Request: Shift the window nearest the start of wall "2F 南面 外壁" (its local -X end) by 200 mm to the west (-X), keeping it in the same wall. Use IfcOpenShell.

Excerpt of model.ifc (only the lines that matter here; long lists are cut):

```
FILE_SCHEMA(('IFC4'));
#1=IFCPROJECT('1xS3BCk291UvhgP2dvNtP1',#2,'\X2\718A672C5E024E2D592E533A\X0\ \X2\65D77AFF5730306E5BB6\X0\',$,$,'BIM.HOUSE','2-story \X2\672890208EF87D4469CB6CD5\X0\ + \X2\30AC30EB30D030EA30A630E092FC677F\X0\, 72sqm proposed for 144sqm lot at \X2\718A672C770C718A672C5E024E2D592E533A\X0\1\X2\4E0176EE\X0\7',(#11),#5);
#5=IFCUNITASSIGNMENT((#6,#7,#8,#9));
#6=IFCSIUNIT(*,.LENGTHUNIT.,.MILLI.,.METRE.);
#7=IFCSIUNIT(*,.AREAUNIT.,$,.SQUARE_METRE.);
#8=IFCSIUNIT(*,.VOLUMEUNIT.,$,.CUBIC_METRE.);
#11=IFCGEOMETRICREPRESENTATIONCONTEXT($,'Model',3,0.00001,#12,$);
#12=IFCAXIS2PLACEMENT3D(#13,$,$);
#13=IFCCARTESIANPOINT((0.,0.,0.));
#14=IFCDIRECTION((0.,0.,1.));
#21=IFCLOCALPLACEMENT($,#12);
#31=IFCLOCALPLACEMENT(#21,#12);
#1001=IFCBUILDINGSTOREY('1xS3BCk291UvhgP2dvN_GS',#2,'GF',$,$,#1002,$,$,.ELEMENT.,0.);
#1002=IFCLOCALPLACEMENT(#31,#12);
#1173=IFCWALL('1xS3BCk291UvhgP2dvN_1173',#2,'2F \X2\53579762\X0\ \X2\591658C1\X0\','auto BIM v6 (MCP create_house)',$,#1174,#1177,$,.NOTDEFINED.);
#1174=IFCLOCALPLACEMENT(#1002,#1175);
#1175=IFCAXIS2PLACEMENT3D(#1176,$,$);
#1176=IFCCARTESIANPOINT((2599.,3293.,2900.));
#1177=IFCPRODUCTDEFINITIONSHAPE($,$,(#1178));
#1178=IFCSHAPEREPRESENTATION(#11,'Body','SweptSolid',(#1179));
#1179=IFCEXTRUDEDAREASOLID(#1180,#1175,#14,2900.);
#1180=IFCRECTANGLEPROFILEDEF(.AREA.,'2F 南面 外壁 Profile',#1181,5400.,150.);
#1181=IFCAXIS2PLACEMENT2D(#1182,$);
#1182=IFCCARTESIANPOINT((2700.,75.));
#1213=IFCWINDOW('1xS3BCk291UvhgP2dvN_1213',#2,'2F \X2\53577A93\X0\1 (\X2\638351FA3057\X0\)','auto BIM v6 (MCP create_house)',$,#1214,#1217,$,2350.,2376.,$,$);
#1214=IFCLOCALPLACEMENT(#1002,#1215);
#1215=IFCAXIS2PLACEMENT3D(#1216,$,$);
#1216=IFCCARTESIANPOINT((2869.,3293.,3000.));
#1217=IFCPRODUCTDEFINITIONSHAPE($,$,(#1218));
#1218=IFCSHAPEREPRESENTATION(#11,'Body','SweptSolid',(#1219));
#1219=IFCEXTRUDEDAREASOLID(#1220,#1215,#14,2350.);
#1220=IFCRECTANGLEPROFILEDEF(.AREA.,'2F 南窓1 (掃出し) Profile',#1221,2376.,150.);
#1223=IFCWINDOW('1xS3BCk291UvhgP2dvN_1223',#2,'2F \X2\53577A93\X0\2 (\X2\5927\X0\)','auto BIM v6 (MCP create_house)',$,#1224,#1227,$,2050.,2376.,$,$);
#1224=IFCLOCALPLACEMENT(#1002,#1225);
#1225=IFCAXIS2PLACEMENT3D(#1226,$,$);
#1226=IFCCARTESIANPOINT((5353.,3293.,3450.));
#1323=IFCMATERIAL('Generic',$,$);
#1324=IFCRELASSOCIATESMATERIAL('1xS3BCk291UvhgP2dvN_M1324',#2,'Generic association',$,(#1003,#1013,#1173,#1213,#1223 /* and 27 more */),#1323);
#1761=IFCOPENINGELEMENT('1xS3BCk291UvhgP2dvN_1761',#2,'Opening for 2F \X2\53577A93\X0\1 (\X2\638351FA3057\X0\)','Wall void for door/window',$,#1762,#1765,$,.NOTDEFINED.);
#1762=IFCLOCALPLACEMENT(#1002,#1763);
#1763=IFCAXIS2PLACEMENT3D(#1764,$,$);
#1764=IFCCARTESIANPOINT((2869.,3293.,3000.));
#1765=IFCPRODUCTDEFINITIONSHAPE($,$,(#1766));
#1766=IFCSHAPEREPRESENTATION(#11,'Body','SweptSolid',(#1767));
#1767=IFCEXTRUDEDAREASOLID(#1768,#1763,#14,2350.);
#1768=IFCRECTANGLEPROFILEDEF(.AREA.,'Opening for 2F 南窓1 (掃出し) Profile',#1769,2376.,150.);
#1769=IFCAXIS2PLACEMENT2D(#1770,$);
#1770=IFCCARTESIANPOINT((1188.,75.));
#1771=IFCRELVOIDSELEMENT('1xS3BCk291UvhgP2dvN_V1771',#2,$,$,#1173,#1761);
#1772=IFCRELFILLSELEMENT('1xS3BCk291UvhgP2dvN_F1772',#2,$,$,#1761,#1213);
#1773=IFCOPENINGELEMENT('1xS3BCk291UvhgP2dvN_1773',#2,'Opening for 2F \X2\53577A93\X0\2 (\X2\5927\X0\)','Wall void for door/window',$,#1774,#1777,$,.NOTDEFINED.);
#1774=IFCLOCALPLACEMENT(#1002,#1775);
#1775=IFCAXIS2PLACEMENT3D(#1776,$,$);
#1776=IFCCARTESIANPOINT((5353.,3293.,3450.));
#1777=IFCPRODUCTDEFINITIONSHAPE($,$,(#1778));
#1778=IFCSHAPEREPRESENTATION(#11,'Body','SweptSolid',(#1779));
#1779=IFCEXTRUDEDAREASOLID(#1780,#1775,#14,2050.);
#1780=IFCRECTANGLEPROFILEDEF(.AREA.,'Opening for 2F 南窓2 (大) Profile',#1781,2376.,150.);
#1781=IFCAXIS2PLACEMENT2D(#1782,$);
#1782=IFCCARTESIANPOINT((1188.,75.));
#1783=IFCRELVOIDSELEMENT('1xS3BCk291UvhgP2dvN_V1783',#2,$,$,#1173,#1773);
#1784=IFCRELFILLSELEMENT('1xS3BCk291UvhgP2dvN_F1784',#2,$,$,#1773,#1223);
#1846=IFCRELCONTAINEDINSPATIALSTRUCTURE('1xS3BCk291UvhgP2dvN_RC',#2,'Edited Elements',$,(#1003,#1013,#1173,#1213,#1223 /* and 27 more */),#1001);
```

```python
import ifcopenshell
import ifcopenshell.api.geometry
import ifcopenshell.util.placement

model = ifcopenshell.open("model.ifc")

window = model.by_guid("1xS3BCk291UvhgP2dvN_1213")
opening = window.FillsVoids[0].RelatingOpeningElement
wall = opening.VoidsElements[0].RelatingBuildingElement

wall_matrix = ifcopenshell.util.placement.get_local_placement(wall.ObjectPlacement)
shift = wall_matrix[:3, 0] * -200.0
before = ifcopenshell.util.placement.get_local_placement(window.ObjectPlacement)[:3, 3].copy()

# The window is not placed relative to its opening, so move both.
for product in (opening, window):
    matrix = ifcopenshell.util.placement.get_local_placement(product.ObjectPlacement)
    matrix[:3, 3] += shift
    ifcopenshell.api.geometry.edit_object_placement(model, product=product, matrix=matrix, is_si=False)

after = ifcopenshell.util.placement.get_local_placement(window.ObjectPlacement)[:3, 3]
print("window moved by", (after - before).round(3) + 0.0)

model.write("model_edited.ifc")
```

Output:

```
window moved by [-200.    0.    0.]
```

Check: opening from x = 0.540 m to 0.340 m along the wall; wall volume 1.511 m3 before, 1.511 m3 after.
